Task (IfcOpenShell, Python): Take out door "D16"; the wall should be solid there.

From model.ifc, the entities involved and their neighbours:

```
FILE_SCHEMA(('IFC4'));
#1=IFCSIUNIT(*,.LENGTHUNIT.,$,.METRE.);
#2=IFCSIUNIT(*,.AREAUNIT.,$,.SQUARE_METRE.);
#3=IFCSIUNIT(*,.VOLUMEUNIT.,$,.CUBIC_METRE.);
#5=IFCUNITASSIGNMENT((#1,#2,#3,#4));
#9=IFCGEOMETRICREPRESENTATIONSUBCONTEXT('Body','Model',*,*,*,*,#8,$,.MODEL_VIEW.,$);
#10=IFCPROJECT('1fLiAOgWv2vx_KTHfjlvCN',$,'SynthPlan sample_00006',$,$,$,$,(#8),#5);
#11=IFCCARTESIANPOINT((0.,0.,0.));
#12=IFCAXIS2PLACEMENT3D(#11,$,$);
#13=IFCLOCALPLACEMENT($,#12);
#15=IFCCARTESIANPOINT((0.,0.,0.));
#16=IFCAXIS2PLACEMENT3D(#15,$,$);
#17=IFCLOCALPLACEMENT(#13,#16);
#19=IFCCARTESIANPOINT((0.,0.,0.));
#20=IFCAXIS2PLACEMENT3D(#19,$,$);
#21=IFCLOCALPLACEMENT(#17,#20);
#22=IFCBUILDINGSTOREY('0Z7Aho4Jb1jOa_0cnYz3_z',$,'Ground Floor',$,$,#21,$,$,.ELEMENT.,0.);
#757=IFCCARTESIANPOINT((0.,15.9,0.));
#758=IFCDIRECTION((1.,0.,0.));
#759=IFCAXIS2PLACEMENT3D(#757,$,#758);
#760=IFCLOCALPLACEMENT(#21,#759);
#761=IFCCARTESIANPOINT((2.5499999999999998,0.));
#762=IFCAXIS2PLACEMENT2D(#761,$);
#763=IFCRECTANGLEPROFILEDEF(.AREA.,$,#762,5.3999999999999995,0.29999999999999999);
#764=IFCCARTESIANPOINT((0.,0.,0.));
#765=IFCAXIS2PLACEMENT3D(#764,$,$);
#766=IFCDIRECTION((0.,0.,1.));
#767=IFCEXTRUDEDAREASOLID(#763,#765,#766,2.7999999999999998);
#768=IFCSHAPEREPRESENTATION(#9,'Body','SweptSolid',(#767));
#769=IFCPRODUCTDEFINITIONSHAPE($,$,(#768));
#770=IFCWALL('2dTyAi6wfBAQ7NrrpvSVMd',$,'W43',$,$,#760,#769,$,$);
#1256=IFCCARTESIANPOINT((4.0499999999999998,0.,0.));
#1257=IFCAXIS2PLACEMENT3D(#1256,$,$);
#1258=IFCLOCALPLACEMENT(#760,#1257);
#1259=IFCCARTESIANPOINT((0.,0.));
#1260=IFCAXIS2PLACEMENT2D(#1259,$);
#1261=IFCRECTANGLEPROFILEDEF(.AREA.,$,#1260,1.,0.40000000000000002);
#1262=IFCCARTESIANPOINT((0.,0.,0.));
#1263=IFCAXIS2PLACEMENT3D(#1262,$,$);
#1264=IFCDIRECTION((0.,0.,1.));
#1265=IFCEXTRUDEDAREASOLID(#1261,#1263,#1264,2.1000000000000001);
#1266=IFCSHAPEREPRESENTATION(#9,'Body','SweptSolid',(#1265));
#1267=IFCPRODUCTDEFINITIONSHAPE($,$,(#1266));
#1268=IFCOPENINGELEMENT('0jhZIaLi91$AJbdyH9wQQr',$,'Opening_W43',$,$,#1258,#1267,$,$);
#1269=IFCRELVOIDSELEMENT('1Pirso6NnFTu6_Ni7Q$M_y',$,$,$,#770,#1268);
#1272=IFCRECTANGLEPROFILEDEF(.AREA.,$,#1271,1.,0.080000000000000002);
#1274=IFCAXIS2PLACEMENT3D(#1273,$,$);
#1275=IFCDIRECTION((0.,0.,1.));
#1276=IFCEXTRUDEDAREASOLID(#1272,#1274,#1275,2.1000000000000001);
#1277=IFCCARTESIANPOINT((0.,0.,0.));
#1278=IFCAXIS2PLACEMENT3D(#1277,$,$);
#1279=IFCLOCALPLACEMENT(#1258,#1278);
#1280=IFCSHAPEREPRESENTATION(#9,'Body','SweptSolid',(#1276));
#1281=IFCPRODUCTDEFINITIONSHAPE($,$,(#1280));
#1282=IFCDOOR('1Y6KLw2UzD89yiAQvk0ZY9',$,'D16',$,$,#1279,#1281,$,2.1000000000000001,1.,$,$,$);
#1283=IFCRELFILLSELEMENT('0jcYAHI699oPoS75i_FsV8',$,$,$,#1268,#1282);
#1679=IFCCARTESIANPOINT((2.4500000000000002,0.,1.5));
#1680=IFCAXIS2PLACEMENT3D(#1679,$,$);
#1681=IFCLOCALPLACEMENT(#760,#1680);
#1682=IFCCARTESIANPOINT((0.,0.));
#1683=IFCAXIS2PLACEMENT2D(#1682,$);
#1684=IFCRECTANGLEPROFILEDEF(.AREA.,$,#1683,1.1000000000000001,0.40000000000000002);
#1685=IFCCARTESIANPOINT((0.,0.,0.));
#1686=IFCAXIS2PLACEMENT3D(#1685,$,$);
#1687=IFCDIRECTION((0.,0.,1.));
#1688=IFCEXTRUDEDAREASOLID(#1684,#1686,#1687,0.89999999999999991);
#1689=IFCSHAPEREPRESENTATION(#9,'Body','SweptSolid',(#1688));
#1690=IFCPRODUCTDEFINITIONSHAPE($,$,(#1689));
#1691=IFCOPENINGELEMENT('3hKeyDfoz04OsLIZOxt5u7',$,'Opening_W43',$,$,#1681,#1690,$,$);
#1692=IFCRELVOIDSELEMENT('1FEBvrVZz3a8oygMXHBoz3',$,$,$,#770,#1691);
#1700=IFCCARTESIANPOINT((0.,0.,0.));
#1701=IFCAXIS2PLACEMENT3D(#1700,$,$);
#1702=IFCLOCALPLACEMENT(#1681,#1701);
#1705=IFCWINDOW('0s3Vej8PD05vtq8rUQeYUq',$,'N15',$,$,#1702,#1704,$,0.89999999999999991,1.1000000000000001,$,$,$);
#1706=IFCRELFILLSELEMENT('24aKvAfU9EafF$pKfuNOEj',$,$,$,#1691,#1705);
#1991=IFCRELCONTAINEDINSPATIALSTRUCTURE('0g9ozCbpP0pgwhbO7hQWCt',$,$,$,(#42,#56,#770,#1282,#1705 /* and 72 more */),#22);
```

```python
import ifcopenshell
import ifcopenshell.api.feature
import ifcopenshell.api.root
import ifcopenshell.geom
import ifcopenshell.util.shape

model = ifcopenshell.open("model.ifc")
settings = ifcopenshell.geom.settings()


def volume(element):
    """Net volume in cubic metres, openings subtracted."""
    shape = ifcopenshell.geom.create_shape(settings, element)
    return ifcopenshell.util.shape.get_volume(shape.geometry)


door = model.by_guid("1Y6KLw2UzD89yiAQvk0ZY9")
opening = door.FillsVoids[0].RelatingOpeningElement
wall = opening.VoidsElements[0].RelatingBuildingElement
before = volume(wall)

ifcopenshell.api.root.remove_product(model, product=door)
ifcopenshell.api.feature.remove_feature(model, feature=opening)

after = volume(wall)

print(f"wall volume {before:.3f} -> {after:.3f} m3")

model.write("model_edited.ifc")
```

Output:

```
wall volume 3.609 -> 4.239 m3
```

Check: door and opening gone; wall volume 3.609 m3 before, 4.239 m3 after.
